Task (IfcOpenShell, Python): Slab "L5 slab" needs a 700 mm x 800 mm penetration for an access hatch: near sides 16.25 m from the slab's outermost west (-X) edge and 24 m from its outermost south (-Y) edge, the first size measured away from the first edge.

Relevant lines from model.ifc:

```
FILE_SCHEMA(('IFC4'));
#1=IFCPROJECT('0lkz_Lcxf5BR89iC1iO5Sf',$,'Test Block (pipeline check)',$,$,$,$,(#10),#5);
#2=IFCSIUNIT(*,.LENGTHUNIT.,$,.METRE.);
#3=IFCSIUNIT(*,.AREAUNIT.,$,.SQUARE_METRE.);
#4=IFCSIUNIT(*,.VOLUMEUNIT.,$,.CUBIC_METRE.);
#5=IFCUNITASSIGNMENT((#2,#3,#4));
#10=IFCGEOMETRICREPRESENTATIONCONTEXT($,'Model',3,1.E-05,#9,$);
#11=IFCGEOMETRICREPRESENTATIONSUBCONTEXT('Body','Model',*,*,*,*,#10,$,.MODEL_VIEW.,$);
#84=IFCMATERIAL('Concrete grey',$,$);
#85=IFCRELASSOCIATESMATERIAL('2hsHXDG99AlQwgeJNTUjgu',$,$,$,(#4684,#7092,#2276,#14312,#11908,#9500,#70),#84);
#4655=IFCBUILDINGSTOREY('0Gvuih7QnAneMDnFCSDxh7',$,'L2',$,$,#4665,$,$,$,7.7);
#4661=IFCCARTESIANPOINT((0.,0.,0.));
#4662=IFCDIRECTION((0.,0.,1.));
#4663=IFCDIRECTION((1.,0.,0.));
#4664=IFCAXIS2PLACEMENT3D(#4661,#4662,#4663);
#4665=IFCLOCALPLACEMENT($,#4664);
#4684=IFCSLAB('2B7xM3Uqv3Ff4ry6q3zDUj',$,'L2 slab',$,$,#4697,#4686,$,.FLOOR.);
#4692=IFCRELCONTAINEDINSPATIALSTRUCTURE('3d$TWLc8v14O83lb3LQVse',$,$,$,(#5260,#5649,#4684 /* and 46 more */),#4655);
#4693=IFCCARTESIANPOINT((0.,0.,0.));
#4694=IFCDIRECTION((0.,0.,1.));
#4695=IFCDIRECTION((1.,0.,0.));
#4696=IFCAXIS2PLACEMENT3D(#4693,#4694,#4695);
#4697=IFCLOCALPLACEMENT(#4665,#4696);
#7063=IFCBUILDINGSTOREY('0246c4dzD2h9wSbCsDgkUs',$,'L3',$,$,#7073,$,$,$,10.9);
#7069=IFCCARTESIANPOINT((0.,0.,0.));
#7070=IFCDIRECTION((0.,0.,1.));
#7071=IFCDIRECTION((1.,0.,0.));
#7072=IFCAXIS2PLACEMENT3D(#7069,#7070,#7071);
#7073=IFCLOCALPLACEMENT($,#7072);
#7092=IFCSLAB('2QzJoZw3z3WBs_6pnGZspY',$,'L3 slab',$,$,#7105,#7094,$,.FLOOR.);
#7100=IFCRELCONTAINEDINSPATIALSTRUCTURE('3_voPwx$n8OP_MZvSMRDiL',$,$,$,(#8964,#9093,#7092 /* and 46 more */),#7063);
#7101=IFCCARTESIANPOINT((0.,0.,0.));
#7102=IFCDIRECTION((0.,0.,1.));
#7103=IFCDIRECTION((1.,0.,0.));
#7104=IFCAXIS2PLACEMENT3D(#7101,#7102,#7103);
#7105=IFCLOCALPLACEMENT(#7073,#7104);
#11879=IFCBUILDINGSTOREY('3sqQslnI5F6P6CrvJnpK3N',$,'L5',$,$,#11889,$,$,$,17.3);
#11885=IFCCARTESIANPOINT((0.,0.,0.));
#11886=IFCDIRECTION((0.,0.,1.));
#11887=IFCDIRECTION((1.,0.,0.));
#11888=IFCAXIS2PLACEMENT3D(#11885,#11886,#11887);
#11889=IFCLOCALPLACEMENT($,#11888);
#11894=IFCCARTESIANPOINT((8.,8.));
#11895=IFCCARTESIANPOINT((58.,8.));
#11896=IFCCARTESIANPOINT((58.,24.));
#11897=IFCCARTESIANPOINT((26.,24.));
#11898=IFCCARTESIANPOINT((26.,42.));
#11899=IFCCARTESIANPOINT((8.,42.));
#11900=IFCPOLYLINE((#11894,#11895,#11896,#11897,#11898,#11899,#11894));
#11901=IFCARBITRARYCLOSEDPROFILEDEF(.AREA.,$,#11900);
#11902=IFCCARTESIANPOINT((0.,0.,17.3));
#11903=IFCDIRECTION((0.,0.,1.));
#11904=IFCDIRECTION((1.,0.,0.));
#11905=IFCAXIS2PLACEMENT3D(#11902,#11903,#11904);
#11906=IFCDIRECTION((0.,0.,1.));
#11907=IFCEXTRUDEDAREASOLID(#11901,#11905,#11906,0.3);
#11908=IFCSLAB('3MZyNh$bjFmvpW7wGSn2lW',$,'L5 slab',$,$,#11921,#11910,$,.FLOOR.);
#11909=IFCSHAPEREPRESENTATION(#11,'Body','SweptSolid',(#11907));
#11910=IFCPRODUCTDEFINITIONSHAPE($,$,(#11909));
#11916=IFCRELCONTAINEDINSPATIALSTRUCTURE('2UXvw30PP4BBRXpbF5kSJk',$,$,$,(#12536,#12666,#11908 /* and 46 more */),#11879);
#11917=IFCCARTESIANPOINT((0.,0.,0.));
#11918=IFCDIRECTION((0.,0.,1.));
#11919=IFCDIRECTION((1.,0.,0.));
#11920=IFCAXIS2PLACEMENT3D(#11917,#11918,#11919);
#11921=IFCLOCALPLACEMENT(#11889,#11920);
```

```python
import numpy as np
import ifcopenshell
import ifcopenshell.api.feature
import ifcopenshell.api.geometry
import ifcopenshell.api.root
import ifcopenshell.geom
import ifcopenshell.util.placement
import ifcopenshell.util.representation
import ifcopenshell.util.shape
import ifcopenshell.util.unit

model = ifcopenshell.open("model.ifc")
unit_scale = ifcopenshell.util.unit.calculate_unit_scale(model)
settings = ifcopenshell.geom.settings()


def volume(element):
    """Net volume in cubic metres, openings subtracted."""
    shape = ifcopenshell.geom.create_shape(settings, element)
    return ifcopenshell.util.shape.get_volume(shape.geometry)


slab = model.by_id(11908)
before = volume(slab)

# Extent in the slab's own axes, in metres. The edges named are its -X and -Y sides.
slab_shape = ifcopenshell.geom.create_shape(settings, slab)
vertices = ifcopenshell.util.shape.get_vertices(slab_shape.geometry)
x_min, y_min, bottom = vertices.min(axis=0)
top = vertices[:, 2].max()

opening = ifcopenshell.api.root.create_entity(model, ifc_class="IfcOpeningElement", name="Access hatch opening", predefined_type="OPENING")
context = ifcopenshell.util.representation.get_context(model, "Model", "Body", "MODEL_VIEW")
width, depth = 0.7, 0.8
outline = [(0.0, 0.0), (width, 0.0), (width, depth), (0.0, depth), (0.0, 0.0)]
# Overshoot both faces by 50 mm so the cut is clean.
shape = ifcopenshell.api.geometry.add_slab_representation(
    model, context=context, depth=top - bottom + 0.1, polyline=outline
)
ifcopenshell.api.geometry.assign_representation(model, product=opening, representation=shape)

matrix = ifcopenshell.util.placement.get_local_placement(slab.ObjectPlacement)
matrix[:, 3] = matrix @ np.append(np.array([x_min + 16.25, y_min + 24, bottom - 0.05]) / unit_scale, 1.0)
ifcopenshell.api.geometry.edit_object_placement(model, product=opening, matrix=matrix, is_si=False)
ifcopenshell.api.feature.add_feature(model, feature=opening, element=slab)

after = volume(slab)

print(f"slab volume {before:.3f} -> {after:.3f} m3")

model.write("model_updated.ifc")
```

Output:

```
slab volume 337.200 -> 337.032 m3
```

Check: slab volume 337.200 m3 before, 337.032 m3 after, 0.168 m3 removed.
